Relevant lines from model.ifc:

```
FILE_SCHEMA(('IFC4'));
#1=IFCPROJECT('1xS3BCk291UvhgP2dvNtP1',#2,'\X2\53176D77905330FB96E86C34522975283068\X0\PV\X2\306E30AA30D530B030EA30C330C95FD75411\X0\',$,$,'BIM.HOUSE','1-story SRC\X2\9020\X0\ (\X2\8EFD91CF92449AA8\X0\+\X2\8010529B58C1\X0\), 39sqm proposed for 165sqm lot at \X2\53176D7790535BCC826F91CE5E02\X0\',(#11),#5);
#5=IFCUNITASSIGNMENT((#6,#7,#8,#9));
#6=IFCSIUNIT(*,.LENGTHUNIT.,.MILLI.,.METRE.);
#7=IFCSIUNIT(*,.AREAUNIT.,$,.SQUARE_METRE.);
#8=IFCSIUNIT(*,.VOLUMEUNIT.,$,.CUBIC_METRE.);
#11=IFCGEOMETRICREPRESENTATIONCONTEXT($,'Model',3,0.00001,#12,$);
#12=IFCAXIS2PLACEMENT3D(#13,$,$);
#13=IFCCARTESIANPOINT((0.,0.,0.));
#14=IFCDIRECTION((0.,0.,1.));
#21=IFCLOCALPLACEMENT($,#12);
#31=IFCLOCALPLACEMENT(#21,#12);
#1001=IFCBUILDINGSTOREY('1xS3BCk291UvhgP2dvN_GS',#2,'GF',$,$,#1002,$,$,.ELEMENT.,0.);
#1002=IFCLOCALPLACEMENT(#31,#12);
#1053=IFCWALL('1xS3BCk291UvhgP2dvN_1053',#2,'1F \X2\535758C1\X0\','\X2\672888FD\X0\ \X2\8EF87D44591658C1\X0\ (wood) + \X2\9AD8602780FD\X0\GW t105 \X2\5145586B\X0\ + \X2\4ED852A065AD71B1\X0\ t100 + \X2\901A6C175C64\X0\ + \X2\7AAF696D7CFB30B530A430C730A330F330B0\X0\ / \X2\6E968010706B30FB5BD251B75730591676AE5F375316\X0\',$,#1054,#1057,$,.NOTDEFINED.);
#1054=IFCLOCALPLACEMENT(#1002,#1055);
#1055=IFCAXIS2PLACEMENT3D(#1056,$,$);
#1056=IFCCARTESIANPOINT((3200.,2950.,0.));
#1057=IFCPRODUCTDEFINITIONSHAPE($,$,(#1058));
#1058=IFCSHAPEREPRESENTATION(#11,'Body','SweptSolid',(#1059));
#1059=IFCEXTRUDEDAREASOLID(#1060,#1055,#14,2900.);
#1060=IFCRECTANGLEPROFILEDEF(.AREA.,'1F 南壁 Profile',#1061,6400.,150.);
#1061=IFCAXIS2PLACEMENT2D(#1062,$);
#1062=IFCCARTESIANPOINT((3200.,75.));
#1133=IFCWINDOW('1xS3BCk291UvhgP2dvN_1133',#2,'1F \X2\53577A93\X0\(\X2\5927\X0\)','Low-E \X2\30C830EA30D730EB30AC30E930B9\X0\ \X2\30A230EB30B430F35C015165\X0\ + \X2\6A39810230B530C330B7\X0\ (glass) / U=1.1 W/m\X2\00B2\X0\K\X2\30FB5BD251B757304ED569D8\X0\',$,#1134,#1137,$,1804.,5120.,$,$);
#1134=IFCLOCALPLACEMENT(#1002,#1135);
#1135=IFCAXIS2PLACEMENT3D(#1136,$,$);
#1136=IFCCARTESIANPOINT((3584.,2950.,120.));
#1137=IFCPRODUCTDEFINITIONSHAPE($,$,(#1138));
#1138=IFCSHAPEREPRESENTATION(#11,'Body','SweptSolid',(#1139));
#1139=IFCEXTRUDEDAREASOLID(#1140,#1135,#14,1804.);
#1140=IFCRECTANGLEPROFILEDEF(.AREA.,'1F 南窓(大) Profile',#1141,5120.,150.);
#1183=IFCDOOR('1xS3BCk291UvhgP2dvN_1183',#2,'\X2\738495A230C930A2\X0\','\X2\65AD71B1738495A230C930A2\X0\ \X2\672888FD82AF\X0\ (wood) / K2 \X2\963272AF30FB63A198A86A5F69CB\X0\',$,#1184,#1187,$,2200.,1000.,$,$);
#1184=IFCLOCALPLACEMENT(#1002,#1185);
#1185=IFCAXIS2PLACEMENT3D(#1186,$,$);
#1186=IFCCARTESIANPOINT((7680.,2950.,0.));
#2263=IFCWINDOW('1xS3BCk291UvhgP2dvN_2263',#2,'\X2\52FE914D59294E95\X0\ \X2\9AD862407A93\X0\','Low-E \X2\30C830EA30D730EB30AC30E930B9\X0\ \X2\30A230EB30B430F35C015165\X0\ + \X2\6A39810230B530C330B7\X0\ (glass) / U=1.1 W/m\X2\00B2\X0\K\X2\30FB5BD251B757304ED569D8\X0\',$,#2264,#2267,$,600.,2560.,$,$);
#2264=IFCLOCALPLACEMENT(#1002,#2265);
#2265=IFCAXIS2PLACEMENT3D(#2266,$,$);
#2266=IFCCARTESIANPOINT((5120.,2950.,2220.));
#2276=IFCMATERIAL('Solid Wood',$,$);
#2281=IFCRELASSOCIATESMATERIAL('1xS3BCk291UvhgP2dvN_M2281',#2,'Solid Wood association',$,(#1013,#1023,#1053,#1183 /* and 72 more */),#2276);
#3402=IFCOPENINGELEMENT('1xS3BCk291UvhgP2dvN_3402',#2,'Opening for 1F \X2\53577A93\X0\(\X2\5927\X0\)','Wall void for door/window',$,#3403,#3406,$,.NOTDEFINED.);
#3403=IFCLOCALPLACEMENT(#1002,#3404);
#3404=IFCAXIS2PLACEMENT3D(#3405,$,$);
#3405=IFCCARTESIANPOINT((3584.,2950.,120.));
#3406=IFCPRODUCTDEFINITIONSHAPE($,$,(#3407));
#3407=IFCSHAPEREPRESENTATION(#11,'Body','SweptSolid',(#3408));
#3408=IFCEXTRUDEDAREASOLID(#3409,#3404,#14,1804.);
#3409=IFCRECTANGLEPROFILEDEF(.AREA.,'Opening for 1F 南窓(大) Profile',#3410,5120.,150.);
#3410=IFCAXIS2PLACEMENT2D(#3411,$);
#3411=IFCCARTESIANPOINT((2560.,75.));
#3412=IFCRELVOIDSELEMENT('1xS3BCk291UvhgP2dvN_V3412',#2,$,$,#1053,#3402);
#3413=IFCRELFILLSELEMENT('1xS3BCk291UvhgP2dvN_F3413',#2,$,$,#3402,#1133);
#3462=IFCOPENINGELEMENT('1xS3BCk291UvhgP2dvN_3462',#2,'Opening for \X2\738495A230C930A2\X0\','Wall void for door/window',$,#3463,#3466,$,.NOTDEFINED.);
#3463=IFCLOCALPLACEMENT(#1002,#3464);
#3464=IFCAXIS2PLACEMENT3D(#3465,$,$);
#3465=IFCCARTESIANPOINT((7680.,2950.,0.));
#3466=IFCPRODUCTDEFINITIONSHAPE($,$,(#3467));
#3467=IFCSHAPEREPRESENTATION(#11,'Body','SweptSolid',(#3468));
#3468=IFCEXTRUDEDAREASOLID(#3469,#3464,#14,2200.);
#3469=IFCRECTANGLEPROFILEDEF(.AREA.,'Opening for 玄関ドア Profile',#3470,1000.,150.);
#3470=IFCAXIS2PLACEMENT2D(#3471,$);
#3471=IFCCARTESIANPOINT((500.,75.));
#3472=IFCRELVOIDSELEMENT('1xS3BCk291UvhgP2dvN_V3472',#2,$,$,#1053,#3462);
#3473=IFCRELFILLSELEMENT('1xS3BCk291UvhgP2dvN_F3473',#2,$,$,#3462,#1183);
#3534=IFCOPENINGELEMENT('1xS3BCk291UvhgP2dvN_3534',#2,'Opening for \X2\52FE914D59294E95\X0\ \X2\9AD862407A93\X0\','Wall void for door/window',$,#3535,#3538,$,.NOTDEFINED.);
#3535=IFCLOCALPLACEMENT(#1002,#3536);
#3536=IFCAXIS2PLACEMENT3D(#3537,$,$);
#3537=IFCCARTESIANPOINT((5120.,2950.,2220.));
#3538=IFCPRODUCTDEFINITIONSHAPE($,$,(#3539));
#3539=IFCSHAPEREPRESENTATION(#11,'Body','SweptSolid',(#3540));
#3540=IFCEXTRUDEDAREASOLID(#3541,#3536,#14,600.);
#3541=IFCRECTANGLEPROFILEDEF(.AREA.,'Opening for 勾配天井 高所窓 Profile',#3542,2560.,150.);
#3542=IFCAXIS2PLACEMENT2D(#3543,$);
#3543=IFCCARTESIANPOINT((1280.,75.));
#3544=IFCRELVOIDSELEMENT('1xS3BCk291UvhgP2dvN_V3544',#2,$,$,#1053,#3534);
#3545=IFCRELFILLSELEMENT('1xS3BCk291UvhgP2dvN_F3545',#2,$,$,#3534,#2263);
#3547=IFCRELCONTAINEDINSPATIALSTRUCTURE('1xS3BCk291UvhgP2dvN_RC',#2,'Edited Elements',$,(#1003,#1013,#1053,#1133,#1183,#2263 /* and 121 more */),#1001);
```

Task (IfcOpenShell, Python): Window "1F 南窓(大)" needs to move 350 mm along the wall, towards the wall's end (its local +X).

```python
import ifcopenshell
import ifcopenshell.api.geometry
import ifcopenshell.util.placement
import ifcopenshell.util.unit

model = ifcopenshell.open("model.ifc")
unit_scale = ifcopenshell.util.unit.calculate_unit_scale(model)

window = model.by_guid("1xS3BCk291UvhgP2dvN_1133")
opening = window.FillsVoids[0].RelatingOpeningElement
wall = opening.VoidsElements[0].RelatingBuildingElement

wall_matrix = ifcopenshell.util.placement.get_local_placement(wall.ObjectPlacement)
shift = wall_matrix[:3, 0] * 0.35 / unit_scale
before = ifcopenshell.util.placement.get_local_placement(window.ObjectPlacement)[:3, 3].copy()

# The window is not placed relative to its opening, so move both.
for product in (opening, window):
    matrix = ifcopenshell.util.placement.get_local_placement(product.ObjectPlacement)
    matrix[:3, 3] += shift
    ifcopenshell.api.geometry.edit_object_placement(model, product=product, matrix=matrix, is_si=False)

after = ifcopenshell.util.placement.get_local_placement(window.ObjectPlacement)[:3, 3]
print("window moved by", (after - before).round(3) + 0.0)

model.write("model_updated.ifc")
```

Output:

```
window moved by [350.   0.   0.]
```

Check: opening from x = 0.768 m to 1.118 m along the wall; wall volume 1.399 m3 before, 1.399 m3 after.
